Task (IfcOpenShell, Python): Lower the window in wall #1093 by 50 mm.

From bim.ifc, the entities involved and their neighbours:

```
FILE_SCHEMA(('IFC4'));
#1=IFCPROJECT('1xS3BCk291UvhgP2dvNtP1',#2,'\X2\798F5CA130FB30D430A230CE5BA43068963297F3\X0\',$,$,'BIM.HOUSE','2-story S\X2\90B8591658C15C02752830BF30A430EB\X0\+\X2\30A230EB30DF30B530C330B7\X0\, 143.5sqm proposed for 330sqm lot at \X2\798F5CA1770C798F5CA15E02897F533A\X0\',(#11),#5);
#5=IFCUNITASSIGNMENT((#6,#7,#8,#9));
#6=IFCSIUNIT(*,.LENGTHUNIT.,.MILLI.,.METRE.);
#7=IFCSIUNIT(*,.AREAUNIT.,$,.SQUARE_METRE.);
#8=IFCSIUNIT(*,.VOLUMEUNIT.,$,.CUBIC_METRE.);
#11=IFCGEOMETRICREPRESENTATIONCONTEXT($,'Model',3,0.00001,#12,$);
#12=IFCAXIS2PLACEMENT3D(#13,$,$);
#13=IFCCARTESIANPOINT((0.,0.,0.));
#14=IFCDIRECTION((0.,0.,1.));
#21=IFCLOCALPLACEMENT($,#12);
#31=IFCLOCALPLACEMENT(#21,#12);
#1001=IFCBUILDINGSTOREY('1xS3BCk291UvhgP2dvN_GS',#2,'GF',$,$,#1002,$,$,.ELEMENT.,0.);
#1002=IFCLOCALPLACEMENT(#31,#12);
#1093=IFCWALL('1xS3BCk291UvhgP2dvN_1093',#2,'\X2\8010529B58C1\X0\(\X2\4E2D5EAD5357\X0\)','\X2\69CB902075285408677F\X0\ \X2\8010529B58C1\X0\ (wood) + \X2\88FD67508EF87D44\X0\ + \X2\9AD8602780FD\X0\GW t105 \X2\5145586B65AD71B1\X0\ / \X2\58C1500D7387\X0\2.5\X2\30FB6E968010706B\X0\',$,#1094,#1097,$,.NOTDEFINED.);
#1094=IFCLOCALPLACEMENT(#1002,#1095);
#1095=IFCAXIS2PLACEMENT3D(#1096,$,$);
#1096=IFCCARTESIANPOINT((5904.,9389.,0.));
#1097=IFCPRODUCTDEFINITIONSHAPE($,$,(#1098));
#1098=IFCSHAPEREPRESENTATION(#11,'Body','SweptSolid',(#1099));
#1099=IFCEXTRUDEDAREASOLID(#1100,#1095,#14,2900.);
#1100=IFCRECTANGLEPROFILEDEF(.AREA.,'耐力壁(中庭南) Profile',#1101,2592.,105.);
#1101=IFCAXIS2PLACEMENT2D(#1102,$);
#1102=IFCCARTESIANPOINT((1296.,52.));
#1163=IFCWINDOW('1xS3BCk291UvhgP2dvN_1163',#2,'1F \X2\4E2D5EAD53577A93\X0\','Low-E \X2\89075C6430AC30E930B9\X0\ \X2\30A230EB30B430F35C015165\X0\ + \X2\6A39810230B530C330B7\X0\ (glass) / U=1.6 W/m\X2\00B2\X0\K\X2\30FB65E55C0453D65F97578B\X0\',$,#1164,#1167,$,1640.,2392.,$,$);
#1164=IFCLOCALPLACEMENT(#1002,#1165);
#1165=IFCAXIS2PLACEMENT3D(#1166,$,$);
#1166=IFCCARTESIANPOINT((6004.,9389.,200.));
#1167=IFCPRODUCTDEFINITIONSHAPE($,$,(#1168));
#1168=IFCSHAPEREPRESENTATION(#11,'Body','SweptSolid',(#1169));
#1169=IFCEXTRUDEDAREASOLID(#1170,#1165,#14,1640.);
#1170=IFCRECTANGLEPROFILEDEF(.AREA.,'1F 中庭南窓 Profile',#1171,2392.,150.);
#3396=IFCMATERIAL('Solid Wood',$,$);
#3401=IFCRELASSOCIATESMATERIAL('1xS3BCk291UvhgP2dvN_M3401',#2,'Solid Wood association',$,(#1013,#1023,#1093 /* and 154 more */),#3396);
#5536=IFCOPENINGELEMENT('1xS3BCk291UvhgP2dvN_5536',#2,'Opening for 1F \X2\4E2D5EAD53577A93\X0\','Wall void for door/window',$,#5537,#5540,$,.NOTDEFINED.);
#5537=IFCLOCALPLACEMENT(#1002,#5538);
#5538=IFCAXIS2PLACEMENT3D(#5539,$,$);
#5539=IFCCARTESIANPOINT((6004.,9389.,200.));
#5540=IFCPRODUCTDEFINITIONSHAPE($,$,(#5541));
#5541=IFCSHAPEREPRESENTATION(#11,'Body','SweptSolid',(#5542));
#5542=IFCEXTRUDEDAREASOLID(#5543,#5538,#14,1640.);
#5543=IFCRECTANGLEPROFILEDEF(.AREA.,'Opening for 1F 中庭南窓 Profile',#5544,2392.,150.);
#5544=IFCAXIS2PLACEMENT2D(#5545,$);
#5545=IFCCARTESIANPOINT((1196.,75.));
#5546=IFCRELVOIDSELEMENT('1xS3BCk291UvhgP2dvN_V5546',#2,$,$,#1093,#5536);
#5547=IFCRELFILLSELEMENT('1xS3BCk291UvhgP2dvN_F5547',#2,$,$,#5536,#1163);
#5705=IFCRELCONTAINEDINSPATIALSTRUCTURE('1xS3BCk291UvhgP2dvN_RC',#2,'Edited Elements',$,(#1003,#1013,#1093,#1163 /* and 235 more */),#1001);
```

```python
import numpy as np
import ifcopenshell
import ifcopenshell.api.geometry
import ifcopenshell.util.placement
import ifcopenshell.util.unit

model = ifcopenshell.open("bim.ifc")
unit_scale = ifcopenshell.util.unit.calculate_unit_scale(model)

window = model.by_guid("1xS3BCk291UvhgP2dvN_1163")
opening = window.FillsVoids[0].RelatingOpeningElement
dz = -50.0

shift = np.array([0.0, 0.0, dz])
# The window is not placed relative to its opening, so move both.
for product in (opening, window):
    matrix = ifcopenshell.util.placement.get_local_placement(product.ObjectPlacement)
    matrix[:3, 3] += shift
    ifcopenshell.api.geometry.edit_object_placement(model, product=product, matrix=matrix, is_si=False)

print(f"moved by {dz * unit_scale:+.3f} m")

model.write("bim_rev.ifc")
```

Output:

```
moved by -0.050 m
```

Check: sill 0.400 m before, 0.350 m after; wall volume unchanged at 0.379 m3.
